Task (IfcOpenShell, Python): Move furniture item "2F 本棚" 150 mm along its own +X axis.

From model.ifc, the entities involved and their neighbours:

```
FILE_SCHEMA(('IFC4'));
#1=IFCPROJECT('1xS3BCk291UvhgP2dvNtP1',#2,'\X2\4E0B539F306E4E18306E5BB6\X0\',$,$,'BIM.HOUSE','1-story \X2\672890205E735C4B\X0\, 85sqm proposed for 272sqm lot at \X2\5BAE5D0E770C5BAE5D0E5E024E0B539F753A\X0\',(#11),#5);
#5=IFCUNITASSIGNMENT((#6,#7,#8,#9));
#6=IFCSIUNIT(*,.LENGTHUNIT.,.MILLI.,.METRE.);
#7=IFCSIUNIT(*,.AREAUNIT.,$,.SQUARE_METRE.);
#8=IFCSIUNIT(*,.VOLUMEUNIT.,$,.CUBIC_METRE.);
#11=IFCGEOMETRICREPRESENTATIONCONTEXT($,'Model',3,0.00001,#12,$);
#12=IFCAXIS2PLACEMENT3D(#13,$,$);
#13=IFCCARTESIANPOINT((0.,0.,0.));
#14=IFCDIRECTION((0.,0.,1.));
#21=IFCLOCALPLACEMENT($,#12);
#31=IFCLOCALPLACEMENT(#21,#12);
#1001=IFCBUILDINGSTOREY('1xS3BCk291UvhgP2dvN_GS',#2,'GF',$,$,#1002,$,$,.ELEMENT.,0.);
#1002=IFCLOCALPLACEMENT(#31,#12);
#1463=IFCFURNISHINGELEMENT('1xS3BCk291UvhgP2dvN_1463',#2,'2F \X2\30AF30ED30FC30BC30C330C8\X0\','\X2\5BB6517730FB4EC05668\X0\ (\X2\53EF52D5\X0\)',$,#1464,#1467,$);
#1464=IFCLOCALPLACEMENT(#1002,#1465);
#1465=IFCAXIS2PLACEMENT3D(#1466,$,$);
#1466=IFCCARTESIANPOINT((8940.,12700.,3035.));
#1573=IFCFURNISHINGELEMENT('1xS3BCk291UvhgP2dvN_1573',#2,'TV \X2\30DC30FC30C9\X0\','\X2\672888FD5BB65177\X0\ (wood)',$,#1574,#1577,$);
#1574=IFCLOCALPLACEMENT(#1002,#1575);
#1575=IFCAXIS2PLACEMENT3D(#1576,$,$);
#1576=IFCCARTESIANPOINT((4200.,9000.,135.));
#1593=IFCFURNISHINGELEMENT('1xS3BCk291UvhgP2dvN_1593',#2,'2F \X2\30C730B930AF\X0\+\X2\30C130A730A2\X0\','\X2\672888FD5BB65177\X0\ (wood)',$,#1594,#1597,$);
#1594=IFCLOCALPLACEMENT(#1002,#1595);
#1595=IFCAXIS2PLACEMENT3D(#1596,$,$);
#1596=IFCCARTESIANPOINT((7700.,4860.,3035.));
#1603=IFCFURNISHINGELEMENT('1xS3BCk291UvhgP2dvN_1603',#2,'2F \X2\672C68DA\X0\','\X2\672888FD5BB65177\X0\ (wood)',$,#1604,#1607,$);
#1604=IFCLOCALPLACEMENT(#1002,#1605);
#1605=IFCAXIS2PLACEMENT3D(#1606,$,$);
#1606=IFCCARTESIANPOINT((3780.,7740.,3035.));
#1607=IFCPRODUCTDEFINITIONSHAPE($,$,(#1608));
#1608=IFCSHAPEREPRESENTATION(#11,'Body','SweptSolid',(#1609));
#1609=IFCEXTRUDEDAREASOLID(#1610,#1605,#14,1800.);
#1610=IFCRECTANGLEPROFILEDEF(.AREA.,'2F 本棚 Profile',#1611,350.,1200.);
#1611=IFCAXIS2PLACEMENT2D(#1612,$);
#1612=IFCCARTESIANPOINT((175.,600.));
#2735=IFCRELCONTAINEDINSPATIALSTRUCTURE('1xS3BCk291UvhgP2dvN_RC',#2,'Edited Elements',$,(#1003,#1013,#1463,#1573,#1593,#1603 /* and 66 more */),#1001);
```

```python
import ifcopenshell
import ifcopenshell.api.geometry
import ifcopenshell.util.placement
import ifcopenshell.util.unit

model = ifcopenshell.open("model.ifc")
unit_scale = ifcopenshell.util.unit.calculate_unit_scale(model)

item = model.by_guid("1xS3BCk291UvhgP2dvN_1603")
matrix = ifcopenshell.util.placement.get_local_placement(item.ObjectPlacement)
matrix[:3, 3] += matrix[:3, 0] * 0.15 / unit_scale
ifcopenshell.api.geometry.edit_object_placement(model, product=item, matrix=matrix, is_si=False)

print(ifcopenshell.util.placement.get_local_placement(item.ObjectPlacement).round(3) + 0.0)

model.write("model_updated.ifc")
```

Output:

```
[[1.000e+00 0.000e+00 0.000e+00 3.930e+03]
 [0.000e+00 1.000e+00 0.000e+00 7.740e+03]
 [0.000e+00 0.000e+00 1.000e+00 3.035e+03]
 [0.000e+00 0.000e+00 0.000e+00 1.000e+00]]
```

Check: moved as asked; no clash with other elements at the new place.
